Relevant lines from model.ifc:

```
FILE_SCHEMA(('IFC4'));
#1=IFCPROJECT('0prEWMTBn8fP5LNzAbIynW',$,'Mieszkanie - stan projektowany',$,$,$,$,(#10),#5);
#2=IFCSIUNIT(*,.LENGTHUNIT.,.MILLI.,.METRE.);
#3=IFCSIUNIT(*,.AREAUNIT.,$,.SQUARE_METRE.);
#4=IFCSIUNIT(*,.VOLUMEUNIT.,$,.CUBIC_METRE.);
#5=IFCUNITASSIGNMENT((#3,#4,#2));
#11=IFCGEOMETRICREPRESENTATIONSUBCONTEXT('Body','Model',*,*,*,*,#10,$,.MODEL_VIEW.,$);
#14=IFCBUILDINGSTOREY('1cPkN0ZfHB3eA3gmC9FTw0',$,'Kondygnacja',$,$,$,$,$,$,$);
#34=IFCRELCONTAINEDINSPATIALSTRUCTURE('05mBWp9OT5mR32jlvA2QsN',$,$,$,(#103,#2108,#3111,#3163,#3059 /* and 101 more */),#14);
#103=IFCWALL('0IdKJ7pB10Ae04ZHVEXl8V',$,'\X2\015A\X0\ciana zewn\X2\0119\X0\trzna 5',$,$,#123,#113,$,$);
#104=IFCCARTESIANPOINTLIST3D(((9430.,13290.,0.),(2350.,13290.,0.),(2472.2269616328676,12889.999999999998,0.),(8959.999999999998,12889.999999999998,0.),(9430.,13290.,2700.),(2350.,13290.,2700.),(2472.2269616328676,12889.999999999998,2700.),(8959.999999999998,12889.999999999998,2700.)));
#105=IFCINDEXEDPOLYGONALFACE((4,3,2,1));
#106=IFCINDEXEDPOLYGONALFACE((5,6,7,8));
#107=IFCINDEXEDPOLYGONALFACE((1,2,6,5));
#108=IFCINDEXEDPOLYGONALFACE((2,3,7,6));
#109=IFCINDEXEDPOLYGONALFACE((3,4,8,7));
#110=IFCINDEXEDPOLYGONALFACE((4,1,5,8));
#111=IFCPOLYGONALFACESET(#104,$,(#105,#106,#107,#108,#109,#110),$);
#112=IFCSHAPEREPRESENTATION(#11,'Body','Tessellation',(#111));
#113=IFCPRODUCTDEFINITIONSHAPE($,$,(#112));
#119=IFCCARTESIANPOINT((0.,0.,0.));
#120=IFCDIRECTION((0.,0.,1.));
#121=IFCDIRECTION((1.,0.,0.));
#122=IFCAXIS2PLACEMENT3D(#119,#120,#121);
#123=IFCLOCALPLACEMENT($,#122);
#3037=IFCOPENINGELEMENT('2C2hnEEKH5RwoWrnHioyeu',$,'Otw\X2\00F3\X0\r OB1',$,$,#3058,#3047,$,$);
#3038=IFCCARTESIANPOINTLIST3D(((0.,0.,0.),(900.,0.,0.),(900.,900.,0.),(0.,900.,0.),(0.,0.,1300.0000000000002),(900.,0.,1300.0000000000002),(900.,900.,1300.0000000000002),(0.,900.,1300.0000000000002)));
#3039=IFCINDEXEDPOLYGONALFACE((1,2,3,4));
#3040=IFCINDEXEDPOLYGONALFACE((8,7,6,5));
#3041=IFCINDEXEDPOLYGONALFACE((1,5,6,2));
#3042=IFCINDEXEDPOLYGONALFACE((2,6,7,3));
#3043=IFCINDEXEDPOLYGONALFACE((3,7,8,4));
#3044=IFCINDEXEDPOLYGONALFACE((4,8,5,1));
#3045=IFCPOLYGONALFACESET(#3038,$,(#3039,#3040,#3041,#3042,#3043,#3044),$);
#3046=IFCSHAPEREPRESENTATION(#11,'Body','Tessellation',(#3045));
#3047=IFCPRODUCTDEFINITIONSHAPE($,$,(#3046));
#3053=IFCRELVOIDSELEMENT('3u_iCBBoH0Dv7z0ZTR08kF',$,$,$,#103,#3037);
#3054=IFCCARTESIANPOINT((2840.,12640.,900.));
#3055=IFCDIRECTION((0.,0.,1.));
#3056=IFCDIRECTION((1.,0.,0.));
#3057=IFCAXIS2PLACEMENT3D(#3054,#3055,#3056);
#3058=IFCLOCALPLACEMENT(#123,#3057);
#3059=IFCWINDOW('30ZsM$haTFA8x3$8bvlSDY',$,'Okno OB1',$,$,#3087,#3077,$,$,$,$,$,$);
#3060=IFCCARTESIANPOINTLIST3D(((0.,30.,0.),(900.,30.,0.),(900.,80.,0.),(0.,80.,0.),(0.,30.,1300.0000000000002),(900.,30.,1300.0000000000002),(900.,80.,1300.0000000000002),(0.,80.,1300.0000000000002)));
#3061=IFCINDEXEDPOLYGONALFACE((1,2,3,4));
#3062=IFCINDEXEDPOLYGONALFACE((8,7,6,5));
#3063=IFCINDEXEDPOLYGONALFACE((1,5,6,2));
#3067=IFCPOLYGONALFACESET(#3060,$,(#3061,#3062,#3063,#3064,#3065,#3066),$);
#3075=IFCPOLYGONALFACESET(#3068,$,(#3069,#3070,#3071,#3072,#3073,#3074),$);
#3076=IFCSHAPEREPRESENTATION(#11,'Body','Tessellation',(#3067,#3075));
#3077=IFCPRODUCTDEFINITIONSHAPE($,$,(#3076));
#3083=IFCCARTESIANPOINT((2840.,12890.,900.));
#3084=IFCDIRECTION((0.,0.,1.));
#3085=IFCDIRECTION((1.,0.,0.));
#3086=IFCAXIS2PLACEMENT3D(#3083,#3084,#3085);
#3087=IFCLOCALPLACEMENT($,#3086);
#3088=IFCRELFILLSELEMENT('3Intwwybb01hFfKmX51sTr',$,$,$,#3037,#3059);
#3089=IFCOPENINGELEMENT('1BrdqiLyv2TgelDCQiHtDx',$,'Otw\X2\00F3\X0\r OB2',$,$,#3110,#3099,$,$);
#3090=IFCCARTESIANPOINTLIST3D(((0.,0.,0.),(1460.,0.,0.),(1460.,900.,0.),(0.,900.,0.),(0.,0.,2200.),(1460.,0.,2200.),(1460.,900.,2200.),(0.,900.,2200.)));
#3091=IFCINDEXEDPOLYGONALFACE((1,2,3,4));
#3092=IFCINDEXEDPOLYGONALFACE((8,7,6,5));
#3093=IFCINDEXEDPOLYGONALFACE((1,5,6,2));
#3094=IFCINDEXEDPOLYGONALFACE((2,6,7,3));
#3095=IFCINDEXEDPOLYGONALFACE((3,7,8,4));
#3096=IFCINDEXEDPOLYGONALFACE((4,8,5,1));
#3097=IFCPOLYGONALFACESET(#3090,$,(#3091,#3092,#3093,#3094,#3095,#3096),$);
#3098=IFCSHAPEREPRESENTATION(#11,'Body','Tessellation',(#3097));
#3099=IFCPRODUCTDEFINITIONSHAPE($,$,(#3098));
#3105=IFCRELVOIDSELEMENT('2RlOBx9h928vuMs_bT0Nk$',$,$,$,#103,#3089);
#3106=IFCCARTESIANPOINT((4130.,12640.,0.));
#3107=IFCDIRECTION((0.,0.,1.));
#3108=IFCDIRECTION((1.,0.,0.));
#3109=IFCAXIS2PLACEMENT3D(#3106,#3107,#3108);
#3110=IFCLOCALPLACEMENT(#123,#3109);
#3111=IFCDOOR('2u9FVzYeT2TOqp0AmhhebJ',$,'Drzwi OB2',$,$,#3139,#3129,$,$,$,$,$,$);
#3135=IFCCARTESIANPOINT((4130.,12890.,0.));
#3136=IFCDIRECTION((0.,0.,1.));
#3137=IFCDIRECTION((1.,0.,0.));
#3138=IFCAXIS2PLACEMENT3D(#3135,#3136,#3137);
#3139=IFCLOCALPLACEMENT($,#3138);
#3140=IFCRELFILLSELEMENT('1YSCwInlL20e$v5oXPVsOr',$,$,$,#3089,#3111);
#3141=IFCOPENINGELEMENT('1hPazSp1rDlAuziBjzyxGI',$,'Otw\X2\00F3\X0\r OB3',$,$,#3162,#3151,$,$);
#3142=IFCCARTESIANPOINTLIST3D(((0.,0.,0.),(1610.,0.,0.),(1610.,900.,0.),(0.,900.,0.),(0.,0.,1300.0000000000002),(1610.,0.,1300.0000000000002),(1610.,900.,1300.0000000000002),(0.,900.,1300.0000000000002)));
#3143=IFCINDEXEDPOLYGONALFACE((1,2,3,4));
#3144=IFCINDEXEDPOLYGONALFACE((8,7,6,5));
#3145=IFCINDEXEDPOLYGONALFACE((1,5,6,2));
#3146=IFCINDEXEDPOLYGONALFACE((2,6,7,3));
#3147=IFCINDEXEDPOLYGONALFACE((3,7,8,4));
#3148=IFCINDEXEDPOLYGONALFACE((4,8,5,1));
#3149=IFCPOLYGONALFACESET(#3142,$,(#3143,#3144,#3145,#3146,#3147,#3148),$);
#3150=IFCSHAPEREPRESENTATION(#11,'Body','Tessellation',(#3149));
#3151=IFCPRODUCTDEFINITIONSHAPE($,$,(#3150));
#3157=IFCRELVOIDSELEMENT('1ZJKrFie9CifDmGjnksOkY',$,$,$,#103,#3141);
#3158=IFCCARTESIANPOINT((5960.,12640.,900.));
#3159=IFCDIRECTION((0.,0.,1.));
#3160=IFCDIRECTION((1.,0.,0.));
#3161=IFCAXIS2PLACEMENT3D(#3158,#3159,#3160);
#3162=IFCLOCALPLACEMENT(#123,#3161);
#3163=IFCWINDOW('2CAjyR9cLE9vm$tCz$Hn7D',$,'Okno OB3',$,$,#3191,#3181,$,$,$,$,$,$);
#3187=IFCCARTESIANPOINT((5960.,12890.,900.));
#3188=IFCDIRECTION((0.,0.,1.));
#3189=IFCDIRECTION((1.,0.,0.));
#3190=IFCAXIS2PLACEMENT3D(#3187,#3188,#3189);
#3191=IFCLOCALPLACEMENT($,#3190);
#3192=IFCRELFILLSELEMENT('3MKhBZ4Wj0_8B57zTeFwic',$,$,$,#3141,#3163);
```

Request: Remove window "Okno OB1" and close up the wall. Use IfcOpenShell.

```python
import ifcopenshell
import ifcopenshell.api.feature
import ifcopenshell.api.root
import ifcopenshell.geom
import ifcopenshell.util.shape

model = ifcopenshell.open("model.ifc")
settings = ifcopenshell.geom.settings()


def volume(element):
    """Net volume in cubic metres, openings subtracted."""
    shape = ifcopenshell.geom.create_shape(settings, element)
    return ifcopenshell.util.shape.get_volume(shape.geometry)


window = model.by_guid("30ZsM$haTFA8x3$8bvlSDY")
opening = window.FillsVoids[0].RelatingOpeningElement
wall = opening.VoidsElements[0].RelatingBuildingElement
before = volume(wall)

ifcopenshell.api.root.remove_product(model, product=window)
ifcopenshell.api.feature.remove_feature(model, feature=opening)

after = volume(wall)

print(f"wall volume {before:.3f} -> {after:.3f} m3")

model.write("model_rev.ifc")
```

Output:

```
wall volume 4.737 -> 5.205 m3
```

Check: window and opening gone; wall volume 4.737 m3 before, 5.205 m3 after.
